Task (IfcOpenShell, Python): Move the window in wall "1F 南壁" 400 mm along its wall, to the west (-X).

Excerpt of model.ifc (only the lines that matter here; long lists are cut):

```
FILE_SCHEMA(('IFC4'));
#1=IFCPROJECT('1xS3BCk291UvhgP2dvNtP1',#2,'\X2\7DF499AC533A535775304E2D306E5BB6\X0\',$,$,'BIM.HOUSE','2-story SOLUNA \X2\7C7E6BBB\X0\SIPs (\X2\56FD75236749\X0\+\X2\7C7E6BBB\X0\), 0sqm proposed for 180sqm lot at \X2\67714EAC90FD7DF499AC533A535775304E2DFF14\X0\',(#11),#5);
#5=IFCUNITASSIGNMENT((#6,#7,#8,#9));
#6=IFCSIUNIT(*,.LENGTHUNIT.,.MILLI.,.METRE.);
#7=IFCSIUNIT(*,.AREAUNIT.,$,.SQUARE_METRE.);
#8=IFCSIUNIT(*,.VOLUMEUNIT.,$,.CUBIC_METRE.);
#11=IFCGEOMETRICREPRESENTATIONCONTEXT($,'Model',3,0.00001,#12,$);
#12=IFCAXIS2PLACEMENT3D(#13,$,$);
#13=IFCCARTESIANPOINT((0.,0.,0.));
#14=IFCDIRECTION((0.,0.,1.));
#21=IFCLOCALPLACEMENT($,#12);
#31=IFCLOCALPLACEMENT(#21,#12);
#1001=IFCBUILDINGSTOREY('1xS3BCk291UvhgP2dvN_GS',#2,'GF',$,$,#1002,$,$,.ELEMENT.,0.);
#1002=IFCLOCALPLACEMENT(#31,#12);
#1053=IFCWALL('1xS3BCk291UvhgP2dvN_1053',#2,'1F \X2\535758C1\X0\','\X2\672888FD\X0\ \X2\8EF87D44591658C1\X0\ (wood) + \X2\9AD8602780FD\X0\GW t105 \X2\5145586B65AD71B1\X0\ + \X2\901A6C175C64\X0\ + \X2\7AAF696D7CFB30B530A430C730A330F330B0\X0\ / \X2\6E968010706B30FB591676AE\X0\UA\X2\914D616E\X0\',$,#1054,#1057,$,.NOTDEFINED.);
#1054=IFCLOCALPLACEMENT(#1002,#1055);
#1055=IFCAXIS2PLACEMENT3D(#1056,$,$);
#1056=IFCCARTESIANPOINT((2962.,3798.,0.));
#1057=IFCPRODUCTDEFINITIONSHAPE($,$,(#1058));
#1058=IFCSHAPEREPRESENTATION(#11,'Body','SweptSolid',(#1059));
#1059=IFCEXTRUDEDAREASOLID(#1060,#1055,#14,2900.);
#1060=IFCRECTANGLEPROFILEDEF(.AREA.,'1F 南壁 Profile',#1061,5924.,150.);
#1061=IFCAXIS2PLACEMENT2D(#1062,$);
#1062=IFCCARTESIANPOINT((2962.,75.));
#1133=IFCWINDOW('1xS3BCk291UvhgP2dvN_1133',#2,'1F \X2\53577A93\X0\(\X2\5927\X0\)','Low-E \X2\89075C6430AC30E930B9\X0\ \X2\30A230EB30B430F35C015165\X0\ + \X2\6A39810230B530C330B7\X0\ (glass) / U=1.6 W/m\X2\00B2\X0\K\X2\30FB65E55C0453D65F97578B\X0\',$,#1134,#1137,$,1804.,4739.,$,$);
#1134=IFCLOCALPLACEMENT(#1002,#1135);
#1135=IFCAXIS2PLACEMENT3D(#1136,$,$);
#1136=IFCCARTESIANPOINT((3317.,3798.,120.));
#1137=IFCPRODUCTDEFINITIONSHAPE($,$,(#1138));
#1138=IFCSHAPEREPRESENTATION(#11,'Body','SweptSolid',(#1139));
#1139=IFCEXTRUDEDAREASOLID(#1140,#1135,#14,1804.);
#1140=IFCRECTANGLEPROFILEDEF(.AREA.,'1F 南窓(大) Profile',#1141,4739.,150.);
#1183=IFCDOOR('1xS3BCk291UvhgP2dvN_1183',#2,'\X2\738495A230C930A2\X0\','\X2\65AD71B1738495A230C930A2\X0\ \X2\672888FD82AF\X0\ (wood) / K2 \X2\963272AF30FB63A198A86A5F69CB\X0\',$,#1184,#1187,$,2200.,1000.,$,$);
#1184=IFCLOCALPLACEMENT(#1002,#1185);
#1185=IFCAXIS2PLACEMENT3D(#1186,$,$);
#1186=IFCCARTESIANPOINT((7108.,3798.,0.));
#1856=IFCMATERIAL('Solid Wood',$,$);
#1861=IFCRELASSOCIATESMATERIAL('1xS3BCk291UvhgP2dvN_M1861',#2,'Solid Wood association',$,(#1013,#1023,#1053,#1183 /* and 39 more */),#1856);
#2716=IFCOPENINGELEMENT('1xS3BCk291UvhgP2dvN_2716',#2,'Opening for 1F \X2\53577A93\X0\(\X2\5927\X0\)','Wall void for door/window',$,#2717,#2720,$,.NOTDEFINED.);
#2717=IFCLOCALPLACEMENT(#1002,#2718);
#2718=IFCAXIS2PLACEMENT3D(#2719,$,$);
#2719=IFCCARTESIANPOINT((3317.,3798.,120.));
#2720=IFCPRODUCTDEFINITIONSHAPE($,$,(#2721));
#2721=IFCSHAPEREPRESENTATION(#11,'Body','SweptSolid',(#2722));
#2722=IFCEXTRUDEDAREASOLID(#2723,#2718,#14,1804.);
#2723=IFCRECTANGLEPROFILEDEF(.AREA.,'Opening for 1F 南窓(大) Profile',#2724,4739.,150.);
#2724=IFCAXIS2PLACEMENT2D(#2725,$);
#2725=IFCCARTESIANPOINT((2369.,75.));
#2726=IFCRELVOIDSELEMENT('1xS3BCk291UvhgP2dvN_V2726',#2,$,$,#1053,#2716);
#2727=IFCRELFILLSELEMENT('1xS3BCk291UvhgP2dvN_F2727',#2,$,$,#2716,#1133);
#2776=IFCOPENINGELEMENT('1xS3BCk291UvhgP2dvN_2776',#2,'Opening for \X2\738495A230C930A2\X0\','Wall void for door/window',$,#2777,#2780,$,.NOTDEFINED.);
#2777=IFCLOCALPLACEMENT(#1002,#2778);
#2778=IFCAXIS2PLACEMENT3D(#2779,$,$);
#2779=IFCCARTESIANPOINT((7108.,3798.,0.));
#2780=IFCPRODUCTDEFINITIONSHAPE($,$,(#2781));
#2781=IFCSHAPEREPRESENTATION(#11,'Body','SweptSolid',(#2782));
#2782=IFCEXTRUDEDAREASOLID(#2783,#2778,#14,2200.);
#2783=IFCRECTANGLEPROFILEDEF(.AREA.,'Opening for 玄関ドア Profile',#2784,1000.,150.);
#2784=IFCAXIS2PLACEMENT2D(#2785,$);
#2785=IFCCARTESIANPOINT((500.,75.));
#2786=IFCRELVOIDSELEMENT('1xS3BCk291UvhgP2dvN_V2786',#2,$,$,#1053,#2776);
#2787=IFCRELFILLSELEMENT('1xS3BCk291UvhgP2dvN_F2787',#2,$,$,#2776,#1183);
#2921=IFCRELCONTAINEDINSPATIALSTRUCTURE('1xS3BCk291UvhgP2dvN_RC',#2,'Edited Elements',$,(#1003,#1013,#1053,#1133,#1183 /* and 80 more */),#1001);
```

```python
import ifcopenshell
import ifcopenshell.api.geometry
import ifcopenshell.util.placement
import ifcopenshell.util.unit

model = ifcopenshell.open("model.ifc")
unit_scale = ifcopenshell.util.unit.calculate_unit_scale(model)

window = model.by_id(1133)
opening = window.FillsVoids[0].RelatingOpeningElement
wall = opening.VoidsElements[0].RelatingBuildingElement

wall_matrix = ifcopenshell.util.placement.get_local_placement(wall.ObjectPlacement)
shift = wall_matrix[:3, 0] * -0.4 / unit_scale
before = ifcopenshell.util.placement.get_local_placement(window.ObjectPlacement)[:3, 3].copy()

# The window is not placed relative to its opening, so move both.
for product in (opening, window):
    matrix = ifcopenshell.util.placement.get_local_placement(product.ObjectPlacement)
    matrix[:3, 3] += shift
    ifcopenshell.api.geometry.edit_object_placement(model, product=product, matrix=matrix, is_si=False)

after = ifcopenshell.util.placement.get_local_placement(window.ObjectPlacement)[:3, 3]
print("window moved by", (after - before).round(3) + 0.0)

model.write("model_updated.ifc")
```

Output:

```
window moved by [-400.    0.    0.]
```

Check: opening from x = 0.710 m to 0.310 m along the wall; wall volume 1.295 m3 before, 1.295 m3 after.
